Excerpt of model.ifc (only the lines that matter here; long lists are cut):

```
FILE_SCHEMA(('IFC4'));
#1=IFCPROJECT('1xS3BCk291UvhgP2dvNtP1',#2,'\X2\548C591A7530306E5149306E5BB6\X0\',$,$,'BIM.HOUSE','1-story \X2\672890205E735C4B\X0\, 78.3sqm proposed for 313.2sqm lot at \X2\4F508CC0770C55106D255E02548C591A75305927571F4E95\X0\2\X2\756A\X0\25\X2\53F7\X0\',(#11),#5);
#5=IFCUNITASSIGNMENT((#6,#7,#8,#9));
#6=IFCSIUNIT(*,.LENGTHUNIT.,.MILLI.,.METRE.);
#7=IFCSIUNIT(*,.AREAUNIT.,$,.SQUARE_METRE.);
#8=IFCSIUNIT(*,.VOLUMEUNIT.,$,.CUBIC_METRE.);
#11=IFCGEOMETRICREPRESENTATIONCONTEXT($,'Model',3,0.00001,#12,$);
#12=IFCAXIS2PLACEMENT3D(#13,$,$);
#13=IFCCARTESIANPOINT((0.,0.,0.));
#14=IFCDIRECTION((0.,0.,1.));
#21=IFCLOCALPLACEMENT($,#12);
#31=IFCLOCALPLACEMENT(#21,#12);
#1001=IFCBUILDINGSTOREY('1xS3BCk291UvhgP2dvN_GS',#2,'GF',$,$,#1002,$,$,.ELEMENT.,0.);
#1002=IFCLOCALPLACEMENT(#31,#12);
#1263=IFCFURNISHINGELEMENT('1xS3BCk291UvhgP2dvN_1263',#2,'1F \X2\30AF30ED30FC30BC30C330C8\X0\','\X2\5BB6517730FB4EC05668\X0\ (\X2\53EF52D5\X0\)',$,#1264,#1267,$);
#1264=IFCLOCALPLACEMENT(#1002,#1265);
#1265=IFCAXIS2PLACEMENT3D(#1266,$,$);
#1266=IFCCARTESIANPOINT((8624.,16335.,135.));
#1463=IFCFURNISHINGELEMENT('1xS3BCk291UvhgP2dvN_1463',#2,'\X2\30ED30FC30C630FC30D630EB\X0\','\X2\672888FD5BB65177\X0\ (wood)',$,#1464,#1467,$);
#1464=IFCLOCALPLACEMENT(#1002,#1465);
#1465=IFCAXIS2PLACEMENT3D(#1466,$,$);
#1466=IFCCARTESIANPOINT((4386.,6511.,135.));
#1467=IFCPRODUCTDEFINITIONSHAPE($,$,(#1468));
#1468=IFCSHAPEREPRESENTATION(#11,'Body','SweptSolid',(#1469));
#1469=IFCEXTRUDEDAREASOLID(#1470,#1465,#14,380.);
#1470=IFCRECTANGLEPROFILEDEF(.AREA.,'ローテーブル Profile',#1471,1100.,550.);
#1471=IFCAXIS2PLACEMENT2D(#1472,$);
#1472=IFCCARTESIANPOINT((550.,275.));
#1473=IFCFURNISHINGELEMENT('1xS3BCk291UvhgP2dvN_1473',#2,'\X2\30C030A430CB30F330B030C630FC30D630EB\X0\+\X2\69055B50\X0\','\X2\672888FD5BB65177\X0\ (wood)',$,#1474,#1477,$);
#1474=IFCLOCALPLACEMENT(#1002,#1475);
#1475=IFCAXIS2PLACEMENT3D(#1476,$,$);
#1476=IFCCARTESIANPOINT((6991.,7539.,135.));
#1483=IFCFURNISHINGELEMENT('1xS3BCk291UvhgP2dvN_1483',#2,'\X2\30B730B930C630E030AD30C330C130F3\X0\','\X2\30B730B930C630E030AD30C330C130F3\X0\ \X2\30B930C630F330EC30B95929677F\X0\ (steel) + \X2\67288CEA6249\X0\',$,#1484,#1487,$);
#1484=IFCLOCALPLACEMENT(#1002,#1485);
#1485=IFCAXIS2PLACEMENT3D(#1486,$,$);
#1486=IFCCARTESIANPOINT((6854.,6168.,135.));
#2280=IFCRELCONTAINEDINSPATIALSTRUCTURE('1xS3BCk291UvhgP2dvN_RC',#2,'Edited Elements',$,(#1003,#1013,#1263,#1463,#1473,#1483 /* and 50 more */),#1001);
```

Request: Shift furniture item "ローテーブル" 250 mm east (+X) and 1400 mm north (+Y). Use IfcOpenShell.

```python
import ifcopenshell
import ifcopenshell.api.geometry
import ifcopenshell.util.placement
import ifcopenshell.util.unit

model = ifcopenshell.open("model.ifc")
unit_scale = ifcopenshell.util.unit.calculate_unit_scale(model)

item = model.by_guid("1xS3BCk291UvhgP2dvN_1463")
matrix = ifcopenshell.util.placement.get_local_placement(item.ObjectPlacement)
matrix[0, 3] += 0.25 / unit_scale
matrix[1, 3] += 1.4 / unit_scale
ifcopenshell.api.geometry.edit_object_placement(model, product=item, matrix=matrix, is_si=False)

print(ifcopenshell.util.placement.get_local_placement(item.ObjectPlacement).round(3) + 0.0)

model.write("model_rev.ifc")
```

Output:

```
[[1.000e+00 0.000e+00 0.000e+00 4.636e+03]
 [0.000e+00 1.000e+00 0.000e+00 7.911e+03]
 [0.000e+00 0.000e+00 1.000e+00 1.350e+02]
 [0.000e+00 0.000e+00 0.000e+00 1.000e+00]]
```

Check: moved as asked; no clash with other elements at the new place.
